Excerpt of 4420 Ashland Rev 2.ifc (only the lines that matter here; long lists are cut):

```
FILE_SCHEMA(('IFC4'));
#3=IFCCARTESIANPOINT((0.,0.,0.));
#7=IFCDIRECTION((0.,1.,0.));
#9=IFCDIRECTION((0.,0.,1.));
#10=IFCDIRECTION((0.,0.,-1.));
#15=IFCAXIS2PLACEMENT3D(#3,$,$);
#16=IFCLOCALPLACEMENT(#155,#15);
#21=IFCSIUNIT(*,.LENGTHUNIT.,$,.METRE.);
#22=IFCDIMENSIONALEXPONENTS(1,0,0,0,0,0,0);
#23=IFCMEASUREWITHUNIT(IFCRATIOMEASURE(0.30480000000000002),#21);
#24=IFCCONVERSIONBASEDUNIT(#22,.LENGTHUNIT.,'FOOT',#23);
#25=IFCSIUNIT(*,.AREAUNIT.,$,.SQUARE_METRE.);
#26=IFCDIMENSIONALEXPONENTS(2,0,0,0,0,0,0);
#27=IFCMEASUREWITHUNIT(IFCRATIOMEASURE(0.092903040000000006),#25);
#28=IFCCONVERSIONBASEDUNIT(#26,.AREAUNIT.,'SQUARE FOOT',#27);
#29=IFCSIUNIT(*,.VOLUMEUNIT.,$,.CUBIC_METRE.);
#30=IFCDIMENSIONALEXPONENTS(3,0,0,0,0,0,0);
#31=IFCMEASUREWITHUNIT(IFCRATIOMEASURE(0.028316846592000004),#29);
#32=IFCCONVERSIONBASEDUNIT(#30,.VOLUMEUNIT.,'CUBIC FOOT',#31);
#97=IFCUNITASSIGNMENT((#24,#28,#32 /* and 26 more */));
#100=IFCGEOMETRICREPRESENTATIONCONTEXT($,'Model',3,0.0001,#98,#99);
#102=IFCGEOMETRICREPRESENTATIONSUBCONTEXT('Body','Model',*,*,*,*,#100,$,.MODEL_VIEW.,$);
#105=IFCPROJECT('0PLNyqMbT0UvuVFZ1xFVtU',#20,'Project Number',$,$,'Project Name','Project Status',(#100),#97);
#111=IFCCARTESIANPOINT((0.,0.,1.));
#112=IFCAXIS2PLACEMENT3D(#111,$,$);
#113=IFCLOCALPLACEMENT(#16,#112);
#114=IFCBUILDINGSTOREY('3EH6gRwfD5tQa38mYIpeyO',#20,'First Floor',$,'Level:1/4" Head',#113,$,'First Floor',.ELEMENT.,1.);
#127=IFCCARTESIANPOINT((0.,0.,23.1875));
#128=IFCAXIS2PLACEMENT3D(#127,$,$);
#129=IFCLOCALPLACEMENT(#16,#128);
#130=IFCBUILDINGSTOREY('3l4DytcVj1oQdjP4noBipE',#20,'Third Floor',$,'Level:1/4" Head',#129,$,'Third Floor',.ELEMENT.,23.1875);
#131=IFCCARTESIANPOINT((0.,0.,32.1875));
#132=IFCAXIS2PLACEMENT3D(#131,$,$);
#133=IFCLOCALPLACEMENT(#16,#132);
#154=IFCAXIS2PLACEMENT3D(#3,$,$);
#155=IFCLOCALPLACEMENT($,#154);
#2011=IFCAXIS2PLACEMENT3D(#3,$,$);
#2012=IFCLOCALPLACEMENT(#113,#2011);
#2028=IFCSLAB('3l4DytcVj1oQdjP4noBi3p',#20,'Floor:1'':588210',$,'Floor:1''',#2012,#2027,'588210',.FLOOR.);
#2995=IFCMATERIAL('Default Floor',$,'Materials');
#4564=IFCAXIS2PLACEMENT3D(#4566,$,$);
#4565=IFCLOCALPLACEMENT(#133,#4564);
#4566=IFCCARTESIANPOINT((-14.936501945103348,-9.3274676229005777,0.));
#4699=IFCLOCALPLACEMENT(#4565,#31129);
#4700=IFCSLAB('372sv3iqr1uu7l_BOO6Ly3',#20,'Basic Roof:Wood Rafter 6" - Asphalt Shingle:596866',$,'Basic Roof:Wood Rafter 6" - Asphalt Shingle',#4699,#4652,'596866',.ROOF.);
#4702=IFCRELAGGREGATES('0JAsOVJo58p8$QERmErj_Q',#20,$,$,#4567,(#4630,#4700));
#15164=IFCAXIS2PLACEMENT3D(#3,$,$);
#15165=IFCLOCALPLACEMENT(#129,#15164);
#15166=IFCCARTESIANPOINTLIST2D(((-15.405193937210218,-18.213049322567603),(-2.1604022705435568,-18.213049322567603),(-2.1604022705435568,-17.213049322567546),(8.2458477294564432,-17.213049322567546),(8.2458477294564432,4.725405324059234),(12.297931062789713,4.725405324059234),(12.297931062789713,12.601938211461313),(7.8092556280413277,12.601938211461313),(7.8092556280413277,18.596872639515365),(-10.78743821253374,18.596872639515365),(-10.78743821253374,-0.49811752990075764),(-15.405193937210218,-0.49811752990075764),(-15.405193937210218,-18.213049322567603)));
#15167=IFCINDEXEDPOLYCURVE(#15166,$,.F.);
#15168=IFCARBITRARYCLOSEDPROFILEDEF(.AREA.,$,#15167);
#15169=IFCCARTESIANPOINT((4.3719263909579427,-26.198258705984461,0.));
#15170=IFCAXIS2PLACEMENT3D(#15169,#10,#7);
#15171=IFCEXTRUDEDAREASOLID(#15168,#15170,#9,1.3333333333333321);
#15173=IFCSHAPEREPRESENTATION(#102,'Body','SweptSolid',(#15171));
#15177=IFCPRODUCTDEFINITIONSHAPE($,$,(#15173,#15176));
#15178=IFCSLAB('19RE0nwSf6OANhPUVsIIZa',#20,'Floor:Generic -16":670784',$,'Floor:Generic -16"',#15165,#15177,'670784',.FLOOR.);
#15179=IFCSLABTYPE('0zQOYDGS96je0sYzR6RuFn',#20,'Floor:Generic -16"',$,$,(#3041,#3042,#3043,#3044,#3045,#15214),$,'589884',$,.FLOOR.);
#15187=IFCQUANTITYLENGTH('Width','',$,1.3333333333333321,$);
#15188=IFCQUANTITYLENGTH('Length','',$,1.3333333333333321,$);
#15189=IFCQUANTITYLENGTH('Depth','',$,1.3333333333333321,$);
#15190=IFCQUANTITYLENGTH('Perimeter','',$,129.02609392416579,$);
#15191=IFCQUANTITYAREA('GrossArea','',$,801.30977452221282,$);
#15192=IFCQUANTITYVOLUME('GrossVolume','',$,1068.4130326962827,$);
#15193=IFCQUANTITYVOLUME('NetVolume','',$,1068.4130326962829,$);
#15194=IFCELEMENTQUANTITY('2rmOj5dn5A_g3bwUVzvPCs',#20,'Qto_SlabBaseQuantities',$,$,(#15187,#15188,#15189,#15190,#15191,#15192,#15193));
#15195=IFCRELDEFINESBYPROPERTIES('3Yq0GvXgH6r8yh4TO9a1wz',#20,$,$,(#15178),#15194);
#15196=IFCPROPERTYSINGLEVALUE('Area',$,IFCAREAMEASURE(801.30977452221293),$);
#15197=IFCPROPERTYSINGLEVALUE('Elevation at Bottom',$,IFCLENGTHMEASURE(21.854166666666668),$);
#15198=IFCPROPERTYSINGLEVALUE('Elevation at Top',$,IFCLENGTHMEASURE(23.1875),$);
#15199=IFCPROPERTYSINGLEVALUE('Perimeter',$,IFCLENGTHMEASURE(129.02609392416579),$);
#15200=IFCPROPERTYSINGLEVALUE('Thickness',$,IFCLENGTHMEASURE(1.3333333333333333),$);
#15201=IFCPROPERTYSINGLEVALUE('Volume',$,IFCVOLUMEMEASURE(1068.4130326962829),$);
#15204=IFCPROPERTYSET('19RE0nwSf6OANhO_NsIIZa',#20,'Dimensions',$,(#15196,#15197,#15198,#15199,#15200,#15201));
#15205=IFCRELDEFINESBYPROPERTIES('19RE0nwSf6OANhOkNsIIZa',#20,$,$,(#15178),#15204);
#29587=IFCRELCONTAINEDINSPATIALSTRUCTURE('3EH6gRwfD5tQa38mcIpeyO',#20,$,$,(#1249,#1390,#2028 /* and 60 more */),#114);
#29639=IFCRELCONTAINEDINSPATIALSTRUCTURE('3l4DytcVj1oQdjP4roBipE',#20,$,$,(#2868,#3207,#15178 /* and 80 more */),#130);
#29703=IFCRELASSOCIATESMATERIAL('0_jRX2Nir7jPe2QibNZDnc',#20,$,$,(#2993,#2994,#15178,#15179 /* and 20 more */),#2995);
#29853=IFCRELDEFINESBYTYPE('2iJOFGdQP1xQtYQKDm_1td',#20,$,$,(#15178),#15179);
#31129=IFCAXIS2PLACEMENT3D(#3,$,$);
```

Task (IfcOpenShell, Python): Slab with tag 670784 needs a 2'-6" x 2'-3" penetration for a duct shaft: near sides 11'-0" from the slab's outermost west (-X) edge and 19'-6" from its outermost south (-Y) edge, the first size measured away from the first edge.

```python
import numpy as np
import ifcopenshell
import ifcopenshell.api.feature
import ifcopenshell.api.geometry
import ifcopenshell.api.pset
import ifcopenshell.api.root
import ifcopenshell.geom
import ifcopenshell.util.element
import ifcopenshell.util.placement
import ifcopenshell.util.representation
import ifcopenshell.util.shape
import ifcopenshell.util.unit

model = ifcopenshell.open("4420 Ashland Rev 2.ifc")
unit_scale = ifcopenshell.util.unit.calculate_unit_scale(model)
area_scale = ifcopenshell.util.unit.calculate_unit_scale(model, "AREAUNIT")
volume_scale = ifcopenshell.util.unit.calculate_unit_scale(model, "VOLUMEUNIT")
settings = ifcopenshell.geom.settings()


def volume(element):
    """Net volume in cubic metres, openings subtracted."""
    shape = ifcopenshell.geom.create_shape(settings, element)
    return ifcopenshell.util.shape.get_volume(shape.geometry)


slab = model.by_guid("19RE0nwSf6OANhPUVsIIZa")
before = volume(slab)

# Extent in the slab's own axes, in metres. The edges named are its -X and -Y sides.
slab_shape = ifcopenshell.geom.create_shape(settings, slab)
vertices = ifcopenshell.util.shape.get_vertices(slab_shape.geometry)
x_min, y_min, bottom = vertices.min(axis=0)
top = vertices[:, 2].max()

opening = ifcopenshell.api.root.create_entity(model, ifc_class="IfcOpeningElement", name="Duct shaft opening", predefined_type="OPENING")
context = ifcopenshell.util.representation.get_context(model, "Model", "Body", "MODEL_VIEW")
width, depth = 0.762, 0.6858
outline = [(0.0, 0.0), (width, 0.0), (width, depth), (0.0, depth), (0.0, 0.0)]
# Overshoot both faces by 50 mm so the cut is clean.
shape = ifcopenshell.api.geometry.add_slab_representation(
    model, context=context, depth=top - bottom + 0.1, polyline=outline
)
ifcopenshell.api.geometry.assign_representation(model, product=opening, representation=shape)

matrix = ifcopenshell.util.placement.get_local_placement(slab.ObjectPlacement)
matrix[:, 3] = matrix @ np.append(np.array([x_min + 3.3528, y_min + 5.9436, bottom - 0.05]) / unit_scale, 1.0)
ifcopenshell.api.geometry.edit_object_placement(model, product=opening, matrix=matrix, is_si=False)
ifcopenshell.api.feature.add_feature(model, feature=opening, element=slab)

after = volume(slab)

# Update the slab's stored quantities.
qto = model.by_id(ifcopenshell.util.element.get_pset(slab, "Qto_SlabBaseQuantities", should_inherit=False)["id"])
ifcopenshell.api.pset.edit_qto(model, qto=qto, properties={"NetVolume": after / volume_scale})
pset = model.by_id(ifcopenshell.util.element.get_pset(slab, "Dimensions", should_inherit=False)["id"])
ifcopenshell.api.pset.edit_pset(model, pset=pset, properties={
    "Area": model.create_entity("IfcAreaMeasure", after / (top - bottom) / area_scale),
    "Volume": model.create_entity("IfcVolumeMeasure", after / volume_scale),
})

print(f"slab volume {before:.3f} -> {after:.3f} m3")

model.write("4420 Ashland Rev 2_updated.ifc")
```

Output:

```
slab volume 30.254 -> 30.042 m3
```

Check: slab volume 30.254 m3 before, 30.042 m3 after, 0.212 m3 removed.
